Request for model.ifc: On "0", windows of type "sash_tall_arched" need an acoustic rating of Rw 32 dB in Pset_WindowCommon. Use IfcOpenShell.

First a look at what the model holds.

```python
import ifcopenshell
import ifcopenshell.util.element

model = ifcopenshell.open("model.ifc")
print(model.schema)
storey = next(s for s in model.by_type("IfcBuildingStorey") if s.Name == "0")
windows = [e for e in ifcopenshell.util.element.get_decomposition(storey) if e.is_a("IfcWindow")]
seen = {}
for e in windows:
    element_type = ifcopenshell.util.element.get_type(e)
    key = (element_type.Name if element_type != e and element_type else None, ifcopenshell.util.element.get_pset(e, "Pset_WindowCommon", "AcousticRating"))
    seen[key] = seen.get(key, 0) + 1
for (name, value), count in sorted(seen.items(), key=str):
    print(count, "x", name, "|", value)
```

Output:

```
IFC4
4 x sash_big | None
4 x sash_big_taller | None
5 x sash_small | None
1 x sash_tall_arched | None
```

```python
import ifcopenshell
import ifcopenshell.api.pset
import ifcopenshell.util.element

model = ifcopenshell.open("model.ifc")

storey = next(s for s in model.by_type("IfcBuildingStorey") if s.Name == "0")
windows = [e for e in ifcopenshell.util.element.get_decomposition(storey) if e.is_a("IfcWindow")]

count = 0
for e in windows:
    element_type = ifcopenshell.util.element.get_type(e)
    if element_type in (None, e) or element_type.Name != "sash_tall_arched":
        continue
    # add_pset returns the element's existing set when there is one.
    pset = ifcopenshell.api.pset.add_pset(model, product=e, name="Pset_WindowCommon")
    ifcopenshell.api.pset.edit_pset(model, pset=pset, properties={"AcousticRating": "Rw 32 dB"})
    count += 1

print(count, "windows updated")

model.write("model_updated.ifc")
```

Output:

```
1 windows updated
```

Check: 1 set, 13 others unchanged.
